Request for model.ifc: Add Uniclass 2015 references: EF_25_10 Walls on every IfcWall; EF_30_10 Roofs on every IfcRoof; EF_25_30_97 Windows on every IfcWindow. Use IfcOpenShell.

First a look at what the model holds.

```python
import ifcopenshell

model = ifcopenshell.open("model.ifc")
print(model.schema)
print("classifications:", [c.Name for c in model.by_type("IfcClassification")])
for ifc_class in ("IfcDoor", "IfcRoof", "IfcStair", "IfcWall", "IfcWindow"):
    print(ifc_class, len(model.by_type(ifc_class)))
```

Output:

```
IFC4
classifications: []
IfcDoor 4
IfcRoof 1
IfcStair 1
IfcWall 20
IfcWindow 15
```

```python
import ifcopenshell
import ifcopenshell.api.classification

model = ifcopenshell.open("model.ifc")

system = ifcopenshell.api.classification.add_classification(model, classification="Uniclass 2015")

codes = {
    "IfcWall": ("EF_25_10", "Walls"),
    "IfcRoof": ("EF_30_10", "Roofs"),
    "IfcWindow": ("EF_25_30_97", "Windows"),
}
for ifc_class, (code, name) in codes.items():
    products = model.by_type(ifc_class)
    ifcopenshell.api.classification.add_reference(
        model, products=products, classification=system, identification=code, name=name
    )
    print(code, len(products))

model.write("model_rev.ifc")
```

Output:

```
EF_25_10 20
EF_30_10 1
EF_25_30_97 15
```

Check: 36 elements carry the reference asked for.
